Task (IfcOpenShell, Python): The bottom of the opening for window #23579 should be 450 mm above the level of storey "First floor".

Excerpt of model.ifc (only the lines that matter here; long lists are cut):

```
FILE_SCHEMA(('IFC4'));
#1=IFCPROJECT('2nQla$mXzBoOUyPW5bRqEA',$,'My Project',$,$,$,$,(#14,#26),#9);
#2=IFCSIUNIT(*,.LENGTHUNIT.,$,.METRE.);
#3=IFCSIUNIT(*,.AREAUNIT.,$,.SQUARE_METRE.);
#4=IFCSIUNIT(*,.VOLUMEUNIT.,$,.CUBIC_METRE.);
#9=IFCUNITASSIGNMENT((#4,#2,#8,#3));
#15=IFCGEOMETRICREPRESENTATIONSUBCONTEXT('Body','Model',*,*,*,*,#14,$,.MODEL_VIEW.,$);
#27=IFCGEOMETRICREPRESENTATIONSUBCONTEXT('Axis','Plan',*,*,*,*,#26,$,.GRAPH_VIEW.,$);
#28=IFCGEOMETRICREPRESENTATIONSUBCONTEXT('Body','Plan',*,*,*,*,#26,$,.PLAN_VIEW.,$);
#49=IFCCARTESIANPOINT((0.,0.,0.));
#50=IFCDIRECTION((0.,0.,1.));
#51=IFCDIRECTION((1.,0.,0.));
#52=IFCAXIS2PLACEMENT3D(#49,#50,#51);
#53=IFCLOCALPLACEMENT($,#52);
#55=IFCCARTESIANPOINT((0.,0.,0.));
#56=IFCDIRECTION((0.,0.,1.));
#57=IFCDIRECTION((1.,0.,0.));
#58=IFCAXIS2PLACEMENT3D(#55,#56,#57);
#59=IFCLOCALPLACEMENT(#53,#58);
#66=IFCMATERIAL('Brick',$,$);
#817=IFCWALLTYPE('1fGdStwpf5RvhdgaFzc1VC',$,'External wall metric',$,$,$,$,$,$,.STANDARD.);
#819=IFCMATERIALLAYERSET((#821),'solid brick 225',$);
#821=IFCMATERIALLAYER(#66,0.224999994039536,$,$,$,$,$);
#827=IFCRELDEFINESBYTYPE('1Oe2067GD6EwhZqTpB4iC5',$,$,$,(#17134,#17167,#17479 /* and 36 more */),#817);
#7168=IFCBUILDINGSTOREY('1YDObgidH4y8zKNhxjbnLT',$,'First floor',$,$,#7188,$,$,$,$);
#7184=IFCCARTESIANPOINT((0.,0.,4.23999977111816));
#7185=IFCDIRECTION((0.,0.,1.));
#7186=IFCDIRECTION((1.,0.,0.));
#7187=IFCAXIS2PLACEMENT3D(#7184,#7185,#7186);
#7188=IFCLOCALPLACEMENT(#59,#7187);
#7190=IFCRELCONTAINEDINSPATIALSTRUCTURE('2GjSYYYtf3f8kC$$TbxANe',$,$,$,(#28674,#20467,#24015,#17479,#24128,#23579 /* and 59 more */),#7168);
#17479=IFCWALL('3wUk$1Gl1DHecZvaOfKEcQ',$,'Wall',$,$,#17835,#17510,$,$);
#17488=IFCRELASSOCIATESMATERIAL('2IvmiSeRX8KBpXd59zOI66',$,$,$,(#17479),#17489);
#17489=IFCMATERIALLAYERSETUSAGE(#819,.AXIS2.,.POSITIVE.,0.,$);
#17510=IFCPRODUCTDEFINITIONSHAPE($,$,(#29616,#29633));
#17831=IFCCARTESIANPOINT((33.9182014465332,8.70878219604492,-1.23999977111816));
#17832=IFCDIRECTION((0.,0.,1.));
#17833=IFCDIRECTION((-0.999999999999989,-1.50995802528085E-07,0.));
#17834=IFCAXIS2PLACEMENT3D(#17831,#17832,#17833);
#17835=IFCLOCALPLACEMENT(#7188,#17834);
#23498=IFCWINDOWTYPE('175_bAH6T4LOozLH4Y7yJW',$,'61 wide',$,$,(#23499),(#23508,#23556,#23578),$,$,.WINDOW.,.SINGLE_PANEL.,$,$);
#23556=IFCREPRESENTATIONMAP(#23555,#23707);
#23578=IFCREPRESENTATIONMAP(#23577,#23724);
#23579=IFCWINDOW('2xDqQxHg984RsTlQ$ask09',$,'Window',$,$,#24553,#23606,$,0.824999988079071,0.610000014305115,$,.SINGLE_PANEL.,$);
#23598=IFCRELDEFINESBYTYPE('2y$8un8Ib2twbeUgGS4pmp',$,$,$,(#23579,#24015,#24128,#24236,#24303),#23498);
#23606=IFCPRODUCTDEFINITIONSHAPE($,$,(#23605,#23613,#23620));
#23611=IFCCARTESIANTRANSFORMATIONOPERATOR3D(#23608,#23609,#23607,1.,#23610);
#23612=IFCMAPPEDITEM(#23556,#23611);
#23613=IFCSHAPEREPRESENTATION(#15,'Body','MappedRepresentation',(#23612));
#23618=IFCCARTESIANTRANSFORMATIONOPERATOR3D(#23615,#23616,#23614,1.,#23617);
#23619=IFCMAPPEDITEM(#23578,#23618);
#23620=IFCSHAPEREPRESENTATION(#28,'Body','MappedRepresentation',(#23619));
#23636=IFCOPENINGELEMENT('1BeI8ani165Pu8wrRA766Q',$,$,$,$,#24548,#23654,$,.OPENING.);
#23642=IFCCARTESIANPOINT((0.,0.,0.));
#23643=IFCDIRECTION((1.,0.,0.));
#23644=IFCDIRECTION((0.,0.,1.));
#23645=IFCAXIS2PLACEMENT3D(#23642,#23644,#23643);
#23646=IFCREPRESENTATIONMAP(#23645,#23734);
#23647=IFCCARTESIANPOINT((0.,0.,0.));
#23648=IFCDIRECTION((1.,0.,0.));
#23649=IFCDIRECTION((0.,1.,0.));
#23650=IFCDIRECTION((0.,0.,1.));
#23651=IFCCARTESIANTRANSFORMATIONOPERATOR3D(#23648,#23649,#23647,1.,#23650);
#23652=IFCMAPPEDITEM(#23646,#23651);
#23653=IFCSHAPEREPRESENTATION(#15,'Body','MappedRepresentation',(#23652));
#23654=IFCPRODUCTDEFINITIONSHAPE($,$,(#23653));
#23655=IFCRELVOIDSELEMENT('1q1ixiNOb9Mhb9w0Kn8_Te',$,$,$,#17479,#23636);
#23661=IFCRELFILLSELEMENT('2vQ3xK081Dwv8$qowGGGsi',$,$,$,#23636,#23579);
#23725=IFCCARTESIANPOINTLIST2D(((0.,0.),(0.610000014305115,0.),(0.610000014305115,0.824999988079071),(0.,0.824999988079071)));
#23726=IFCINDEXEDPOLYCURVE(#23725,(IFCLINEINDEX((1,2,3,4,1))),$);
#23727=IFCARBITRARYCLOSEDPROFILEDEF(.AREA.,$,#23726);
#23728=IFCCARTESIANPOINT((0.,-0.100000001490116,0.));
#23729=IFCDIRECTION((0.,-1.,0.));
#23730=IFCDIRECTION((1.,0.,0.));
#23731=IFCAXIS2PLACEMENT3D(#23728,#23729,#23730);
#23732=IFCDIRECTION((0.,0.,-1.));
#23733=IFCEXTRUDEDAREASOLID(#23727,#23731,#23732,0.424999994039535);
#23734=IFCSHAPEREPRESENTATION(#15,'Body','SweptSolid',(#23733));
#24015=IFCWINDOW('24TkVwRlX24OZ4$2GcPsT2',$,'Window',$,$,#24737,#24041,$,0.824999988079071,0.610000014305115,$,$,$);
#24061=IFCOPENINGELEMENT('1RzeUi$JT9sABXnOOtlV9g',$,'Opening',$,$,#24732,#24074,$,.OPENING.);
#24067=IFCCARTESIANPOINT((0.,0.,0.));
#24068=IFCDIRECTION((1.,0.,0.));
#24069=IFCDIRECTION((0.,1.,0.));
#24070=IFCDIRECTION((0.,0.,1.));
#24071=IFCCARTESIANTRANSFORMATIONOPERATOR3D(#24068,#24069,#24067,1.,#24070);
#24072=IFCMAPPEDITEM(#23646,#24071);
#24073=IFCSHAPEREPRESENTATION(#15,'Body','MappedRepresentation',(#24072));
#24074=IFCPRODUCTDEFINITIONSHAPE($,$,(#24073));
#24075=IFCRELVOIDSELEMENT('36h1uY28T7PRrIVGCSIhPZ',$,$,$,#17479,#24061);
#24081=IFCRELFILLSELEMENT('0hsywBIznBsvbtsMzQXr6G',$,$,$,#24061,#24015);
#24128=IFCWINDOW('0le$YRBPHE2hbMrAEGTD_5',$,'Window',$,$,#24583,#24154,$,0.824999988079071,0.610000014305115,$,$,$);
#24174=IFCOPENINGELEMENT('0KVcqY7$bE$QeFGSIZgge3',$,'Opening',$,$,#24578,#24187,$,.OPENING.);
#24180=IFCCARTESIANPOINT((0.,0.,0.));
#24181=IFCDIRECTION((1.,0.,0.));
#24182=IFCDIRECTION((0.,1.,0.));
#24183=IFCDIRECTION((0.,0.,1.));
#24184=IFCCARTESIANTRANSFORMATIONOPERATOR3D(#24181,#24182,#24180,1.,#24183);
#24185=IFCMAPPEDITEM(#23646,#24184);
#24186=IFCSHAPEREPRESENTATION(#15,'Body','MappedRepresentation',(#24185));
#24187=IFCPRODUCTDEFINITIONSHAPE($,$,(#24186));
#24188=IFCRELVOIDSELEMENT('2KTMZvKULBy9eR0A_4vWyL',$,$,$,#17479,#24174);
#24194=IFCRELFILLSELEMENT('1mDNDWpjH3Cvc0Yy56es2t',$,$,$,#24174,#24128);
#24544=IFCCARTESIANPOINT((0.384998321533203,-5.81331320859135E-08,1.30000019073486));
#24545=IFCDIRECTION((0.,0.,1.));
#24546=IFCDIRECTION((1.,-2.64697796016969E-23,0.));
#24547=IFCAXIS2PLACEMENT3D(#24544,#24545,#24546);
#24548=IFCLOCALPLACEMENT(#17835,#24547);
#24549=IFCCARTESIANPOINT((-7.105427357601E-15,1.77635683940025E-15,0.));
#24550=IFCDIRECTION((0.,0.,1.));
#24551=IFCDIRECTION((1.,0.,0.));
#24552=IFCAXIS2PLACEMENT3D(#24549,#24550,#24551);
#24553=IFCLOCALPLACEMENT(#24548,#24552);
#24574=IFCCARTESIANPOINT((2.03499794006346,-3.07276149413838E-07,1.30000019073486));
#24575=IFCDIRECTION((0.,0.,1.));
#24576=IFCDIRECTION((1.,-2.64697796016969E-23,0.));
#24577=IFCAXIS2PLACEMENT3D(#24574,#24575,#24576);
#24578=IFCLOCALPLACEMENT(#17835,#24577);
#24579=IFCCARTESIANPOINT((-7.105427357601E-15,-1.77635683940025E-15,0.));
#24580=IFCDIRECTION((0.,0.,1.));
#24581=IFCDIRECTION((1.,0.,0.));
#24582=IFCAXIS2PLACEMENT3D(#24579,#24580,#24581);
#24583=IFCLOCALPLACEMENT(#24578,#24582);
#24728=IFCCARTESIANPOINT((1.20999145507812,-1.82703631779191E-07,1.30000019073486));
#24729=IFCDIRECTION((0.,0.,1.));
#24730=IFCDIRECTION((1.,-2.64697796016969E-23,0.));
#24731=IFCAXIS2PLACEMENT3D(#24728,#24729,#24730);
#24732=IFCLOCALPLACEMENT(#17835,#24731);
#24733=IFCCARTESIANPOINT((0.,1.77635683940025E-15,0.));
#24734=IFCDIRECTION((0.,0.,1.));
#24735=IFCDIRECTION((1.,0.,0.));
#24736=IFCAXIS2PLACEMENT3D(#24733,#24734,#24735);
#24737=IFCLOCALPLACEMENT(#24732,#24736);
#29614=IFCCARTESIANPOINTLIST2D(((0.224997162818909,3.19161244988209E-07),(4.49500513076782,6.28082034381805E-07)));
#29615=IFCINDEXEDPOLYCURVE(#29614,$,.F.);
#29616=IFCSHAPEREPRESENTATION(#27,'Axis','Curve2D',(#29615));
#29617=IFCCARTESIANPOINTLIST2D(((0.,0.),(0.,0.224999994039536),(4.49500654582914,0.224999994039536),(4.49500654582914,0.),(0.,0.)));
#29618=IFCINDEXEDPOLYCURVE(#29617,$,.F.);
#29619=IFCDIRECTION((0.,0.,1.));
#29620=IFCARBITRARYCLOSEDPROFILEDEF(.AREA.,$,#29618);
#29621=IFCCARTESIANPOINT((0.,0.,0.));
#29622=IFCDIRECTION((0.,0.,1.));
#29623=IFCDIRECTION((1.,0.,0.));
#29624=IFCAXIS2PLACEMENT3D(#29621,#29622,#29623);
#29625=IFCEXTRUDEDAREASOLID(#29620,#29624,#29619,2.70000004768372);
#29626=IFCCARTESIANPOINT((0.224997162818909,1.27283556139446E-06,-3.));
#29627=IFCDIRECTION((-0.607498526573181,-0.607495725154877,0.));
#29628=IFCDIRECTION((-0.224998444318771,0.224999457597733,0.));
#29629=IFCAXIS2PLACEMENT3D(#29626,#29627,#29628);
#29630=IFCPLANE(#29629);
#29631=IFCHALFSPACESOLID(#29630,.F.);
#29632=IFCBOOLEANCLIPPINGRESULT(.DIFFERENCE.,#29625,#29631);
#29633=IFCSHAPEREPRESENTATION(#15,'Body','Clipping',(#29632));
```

```python
import numpy as np
import ifcopenshell
import ifcopenshell.api.geometry
import ifcopenshell.geom
import ifcopenshell.util.element
import ifcopenshell.util.placement
import ifcopenshell.util.shape
import ifcopenshell.util.unit

model = ifcopenshell.open("model.ifc")
unit_scale = ifcopenshell.util.unit.calculate_unit_scale(model)

window = model.by_guid("2xDqQxHg984RsTlQ$ask09")
opening = window.FillsVoids[0].RelatingOpeningElement
storey = ifcopenshell.util.element.get_container(window, ifc_class="IfcBuildingStorey")
level = ifcopenshell.util.placement.get_local_placement(storey.ObjectPlacement)[2, 3]

# The opening's origin need not be at the sill, so measure its lowest point.
shape = ifcopenshell.geom.create_shape(ifcopenshell.geom.settings(), opening)
bottom = ifcopenshell.util.shape.get_shape_bottom_elevation(shape, shape.geometry) / unit_scale
dz = level + 0.45 - bottom

shift = np.array([0.0, 0.0, dz])
# The window is placed relative to its opening, so it follows when the opening moves.
matrix = ifcopenshell.util.placement.get_local_placement(opening.ObjectPlacement)
matrix[:3, 3] += shift
ifcopenshell.api.geometry.edit_object_placement(
    model, product=opening, matrix=matrix, is_si=False, should_transform_children=True
)

print(f"moved by {dz * unit_scale:+.3f} m")

model.write("model_updated.ifc")
```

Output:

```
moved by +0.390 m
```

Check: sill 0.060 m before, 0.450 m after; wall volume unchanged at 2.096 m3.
